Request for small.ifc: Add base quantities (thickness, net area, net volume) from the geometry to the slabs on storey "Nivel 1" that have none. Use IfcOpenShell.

First a look at what the model holds.

```python
import ifcopenshell
import ifcopenshell.util.element
import ifcopenshell.util.unit

model = ifcopenshell.open("small.ifc")
print(model.schema)
for unit_type in ("LENGTHUNIT", "AREAUNIT", "VOLUMEUNIT"):
    print(unit_type, ifcopenshell.util.unit.calculate_unit_scale(model, unit_type))
storey = next(s for s in model.by_type("IfcBuildingStorey") if s.Name == "Nivel 1")
slabs = [e for e in ifcopenshell.util.element.get_decomposition(storey) if e.is_a("IfcSlab")]
for e in sorted(slabs, key=lambda e: e.id()):
    print(e.id(), e.is_a(), e.Name, list(ifcopenshell.util.element.get_psets(e, qtos_only=True)), sep=" | ")
```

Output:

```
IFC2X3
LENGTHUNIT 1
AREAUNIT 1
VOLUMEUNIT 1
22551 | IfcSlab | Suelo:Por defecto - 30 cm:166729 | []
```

```python
import ifcopenshell
import ifcopenshell.api.pset
import ifcopenshell.geom
import ifcopenshell.util.element
import ifcopenshell.util.shape
import ifcopenshell.util.unit

model = ifcopenshell.open("small.ifc")
unit_scale = ifcopenshell.util.unit.calculate_unit_scale(model)
area_scale = ifcopenshell.util.unit.calculate_unit_scale(model, "AREAUNIT")
volume_scale = ifcopenshell.util.unit.calculate_unit_scale(model, "VOLUMEUNIT")
settings = ifcopenshell.geom.settings()

storey = next(s for s in model.by_type("IfcBuildingStorey") if s.Name == "Nivel 1")
slabs = [e for e in ifcopenshell.util.element.get_decomposition(storey) if e.is_a("IfcSlab")]

for e in sorted(slabs, key=lambda e: e.id()):
    if ifcopenshell.util.element.get_psets(e, qtos_only=True, should_inherit=False):
        continue
    # Geometry comes back in metres, in the element's own axes.
    shape = ifcopenshell.geom.create_shape(settings, e)
    values = {
        "Width": ifcopenshell.util.shape.get_z(shape.geometry) / unit_scale,
        "NetArea": ifcopenshell.util.shape.get_footprint_area(shape.geometry) / area_scale,
        "NetVolume": ifcopenshell.util.shape.get_volume(shape.geometry) / volume_scale,
    }
    qto = ifcopenshell.api.pset.add_qto(model, product=e, name="BaseQuantities")
    ifcopenshell.api.pset.edit_qto(model, qto=qto, properties=values)
    print(e.id(), {k: round(v, 3) for k, v in values.items()})

model.write("small_rev.ifc")
```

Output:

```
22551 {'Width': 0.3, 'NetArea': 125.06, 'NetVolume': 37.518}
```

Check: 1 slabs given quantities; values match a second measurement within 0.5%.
